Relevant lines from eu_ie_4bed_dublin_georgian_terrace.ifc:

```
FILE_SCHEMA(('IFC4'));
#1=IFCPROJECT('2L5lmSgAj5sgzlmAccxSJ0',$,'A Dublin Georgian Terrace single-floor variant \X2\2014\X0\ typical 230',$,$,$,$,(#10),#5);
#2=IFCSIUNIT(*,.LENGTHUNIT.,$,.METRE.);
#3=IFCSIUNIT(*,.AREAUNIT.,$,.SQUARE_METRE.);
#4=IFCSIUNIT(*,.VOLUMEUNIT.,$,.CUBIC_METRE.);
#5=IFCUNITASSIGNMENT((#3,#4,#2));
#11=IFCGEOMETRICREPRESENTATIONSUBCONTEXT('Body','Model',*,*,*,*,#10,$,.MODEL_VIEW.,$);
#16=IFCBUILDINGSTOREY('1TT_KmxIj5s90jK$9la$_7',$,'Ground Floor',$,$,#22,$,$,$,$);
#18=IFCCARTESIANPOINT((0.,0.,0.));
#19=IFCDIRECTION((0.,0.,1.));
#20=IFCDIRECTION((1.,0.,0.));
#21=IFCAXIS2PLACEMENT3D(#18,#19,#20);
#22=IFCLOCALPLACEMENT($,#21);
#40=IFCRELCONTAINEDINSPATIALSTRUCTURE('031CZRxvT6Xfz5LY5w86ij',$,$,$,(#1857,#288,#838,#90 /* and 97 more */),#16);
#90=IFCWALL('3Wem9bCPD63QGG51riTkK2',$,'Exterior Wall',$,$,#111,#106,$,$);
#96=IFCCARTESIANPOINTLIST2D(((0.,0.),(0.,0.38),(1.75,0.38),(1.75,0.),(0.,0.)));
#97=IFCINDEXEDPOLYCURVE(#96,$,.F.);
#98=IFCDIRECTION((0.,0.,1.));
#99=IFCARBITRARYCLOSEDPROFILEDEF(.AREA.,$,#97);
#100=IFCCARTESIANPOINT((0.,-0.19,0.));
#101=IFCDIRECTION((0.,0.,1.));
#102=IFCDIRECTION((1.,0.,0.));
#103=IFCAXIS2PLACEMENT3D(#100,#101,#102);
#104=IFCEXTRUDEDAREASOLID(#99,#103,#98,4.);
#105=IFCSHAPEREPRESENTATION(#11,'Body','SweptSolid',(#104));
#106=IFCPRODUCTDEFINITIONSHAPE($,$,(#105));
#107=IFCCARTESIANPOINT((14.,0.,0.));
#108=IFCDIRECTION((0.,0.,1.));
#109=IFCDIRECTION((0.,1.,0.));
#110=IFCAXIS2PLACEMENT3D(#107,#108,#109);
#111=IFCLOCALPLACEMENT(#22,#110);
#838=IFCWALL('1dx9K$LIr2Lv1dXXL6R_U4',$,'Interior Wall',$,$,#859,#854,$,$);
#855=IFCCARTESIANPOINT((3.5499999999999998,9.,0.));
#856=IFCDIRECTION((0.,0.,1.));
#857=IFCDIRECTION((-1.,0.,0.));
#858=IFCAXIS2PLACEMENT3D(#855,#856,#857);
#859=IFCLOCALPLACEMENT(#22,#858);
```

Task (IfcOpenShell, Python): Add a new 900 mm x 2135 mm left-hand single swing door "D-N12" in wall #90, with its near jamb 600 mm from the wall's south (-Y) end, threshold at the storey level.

```python
import numpy as np
import ifcopenshell
import ifcopenshell.api.feature
import ifcopenshell.api.geometry
import ifcopenshell.api.root
import ifcopenshell.api.spatial
import ifcopenshell.geom
import ifcopenshell.util.element
import ifcopenshell.util.placement
import ifcopenshell.util.representation
import ifcopenshell.util.shape
import ifcopenshell.util.unit

model = ifcopenshell.open("eu_ie_4bed_dublin_georgian_terrace.ifc")
unit_scale = ifcopenshell.util.unit.calculate_unit_scale(model)
settings = ifcopenshell.geom.settings()


def volume(element):
    """Net volume in cubic metres, openings subtracted."""
    shape = ifcopenshell.geom.create_shape(settings, element)
    return ifcopenshell.util.shape.get_volume(shape.geometry)


wall = model.by_guid("3Wem9bCPD63QGG51riTkK2")
storey = ifcopenshell.util.element.get_container(wall, ifc_class="IfcBuildingStorey")
context = ifcopenshell.util.representation.get_context(model, "Model", "Body", "MODEL_VIEW")
before = volume(wall)

width, height, from_end, sill = 0.9, 2.135, 0.6, 0.0  # metres

# The wall runs along its own X axis, and the end named is its -X end.
wall_shape = ifcopenshell.geom.create_shape(settings, wall)
x, y, z = ifcopenshell.util.shape.get_vertices(wall_shape.geometry).T
start = x.min() + from_end
face, thickness = float(y.min()), float(y.max() - y.min())
wall_matrix = ifcopenshell.util.placement.get_local_placement(wall.ObjectPlacement)
level = ifcopenshell.util.placement.get_local_placement(storey.ObjectPlacement)[2, 3]


def in_wall(x, y):
    """Placement at x, y metres in the wall's axes, at sill height."""
    matrix = wall_matrix.copy()
    matrix[:, 3] = wall_matrix @ np.array([x / unit_scale, y / unit_scale, 0.0, 1.0])
    matrix[2, 3] = level + sill / unit_scale
    return matrix


# Opening: a box that overshoots both wall faces by 50 mm.
opening = ifcopenshell.api.root.create_entity(model, ifc_class="IfcOpeningElement", predefined_type="OPENING")
box = ifcopenshell.api.geometry.add_wall_representation(
    model, context=context, length=width, height=height, thickness=thickness + 0.1
)
ifcopenshell.api.geometry.assign_representation(model, product=opening, representation=box)
ifcopenshell.api.geometry.edit_object_placement(model, product=opening, matrix=in_wall(start, face - 0.05), is_si=False)
ifcopenshell.api.feature.add_feature(model, feature=opening, element=wall)

door = ifcopenshell.api.root.create_entity(model, ifc_class="IfcDoor", name="D-N12", predefined_type="DOOR")
door.OverallWidth, door.OverallHeight = width / unit_scale, height / unit_scale
door.OperationType = "SINGLE_SWING_LEFT"
body = ifcopenshell.api.geometry.add_door_representation(
    model,
    context=context,
    overall_width=door.OverallWidth,
    overall_height=door.OverallHeight,
    operation_type="SINGLE_SWING_LEFT",
    lining_properties={"LiningDepth": thickness / unit_scale, "ThresholdDepth": thickness / unit_scale},
)
ifcopenshell.api.geometry.assign_representation(model, product=door, representation=body)
ifcopenshell.api.spatial.assign_container(model, products=[door], relating_structure=storey)
ifcopenshell.api.feature.add_filling(model, opening=opening, element=door)

# The lining spans the wall, so the door starts at the wall face.
ifcopenshell.api.geometry.edit_object_placement(model, product=door, matrix=in_wall(start, face), is_si=False)

after = volume(wall)

print(f"wall volume {before:.3f} -> {after:.3f} m3")

model.write("eu_ie_4bed_dublin_georgian_terrace_rev.ifc")
```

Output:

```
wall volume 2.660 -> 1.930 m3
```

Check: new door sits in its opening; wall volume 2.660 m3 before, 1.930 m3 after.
